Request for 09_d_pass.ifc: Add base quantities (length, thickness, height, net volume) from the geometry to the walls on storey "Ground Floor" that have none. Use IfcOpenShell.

First a look at what the model holds.

```python
import ifcopenshell
import ifcopenshell.util.element
import ifcopenshell.util.unit

model = ifcopenshell.open("09_d_pass.ifc")
print(model.schema)
for unit_type in ("LENGTHUNIT", "AREAUNIT", "VOLUMEUNIT"):
    print(unit_type, ifcopenshell.util.unit.calculate_unit_scale(model, unit_type))
storey = next(s for s in model.by_type("IfcBuildingStorey") if s.Name == "Ground Floor")
walls = [e for e in ifcopenshell.util.element.get_decomposition(storey) if e.is_a("IfcWall")]
for e in sorted(walls, key=lambda e: e.id()):
    print(e.id(), e.is_a(), e.Name, list(ifcopenshell.util.element.get_psets(e, qtos_only=True)), sep=" | ")
```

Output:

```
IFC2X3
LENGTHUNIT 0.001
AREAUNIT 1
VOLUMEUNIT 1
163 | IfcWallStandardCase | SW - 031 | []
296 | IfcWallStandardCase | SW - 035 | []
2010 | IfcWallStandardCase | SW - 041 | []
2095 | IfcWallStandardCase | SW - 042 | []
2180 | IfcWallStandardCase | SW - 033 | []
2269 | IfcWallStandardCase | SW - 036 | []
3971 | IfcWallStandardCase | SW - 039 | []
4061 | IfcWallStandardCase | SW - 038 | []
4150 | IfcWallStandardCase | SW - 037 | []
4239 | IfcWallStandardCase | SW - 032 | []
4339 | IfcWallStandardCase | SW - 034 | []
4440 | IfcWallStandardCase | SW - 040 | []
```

```python
import ifcopenshell
import ifcopenshell.api.pset
import ifcopenshell.geom
import ifcopenshell.util.element
import ifcopenshell.util.shape
import ifcopenshell.util.unit

model = ifcopenshell.open("09_d_pass.ifc")
unit_scale = ifcopenshell.util.unit.calculate_unit_scale(model)
volume_scale = ifcopenshell.util.unit.calculate_unit_scale(model, "VOLUMEUNIT")
settings = ifcopenshell.geom.settings()

storey = next(s for s in model.by_type("IfcBuildingStorey") if s.Name == "Ground Floor")
walls = [e for e in ifcopenshell.util.element.get_decomposition(storey) if e.is_a("IfcWall")]

for e in sorted(walls, key=lambda e: e.id()):
    if ifcopenshell.util.element.get_psets(e, qtos_only=True, should_inherit=False):
        continue
    # Geometry comes back in metres, in the element's own axes.
    shape = ifcopenshell.geom.create_shape(settings, e)
    values = {
        "Length": ifcopenshell.util.shape.get_x(shape.geometry) / unit_scale,
        "Width": ifcopenshell.util.shape.get_y(shape.geometry) / unit_scale,
        "Height": ifcopenshell.util.shape.get_z(shape.geometry) / unit_scale,
        "NetVolume": ifcopenshell.util.shape.get_volume(shape.geometry) / volume_scale,
    }
    qto = ifcopenshell.api.pset.add_qto(model, product=e, name="BaseQuantities")
    ifcopenshell.api.pset.edit_qto(model, qto=qto, properties=values)
    print(e.id(), {k: round(v, 3) for k, v in values.items()})

model.write("09_d_pass_v2.ifc")
```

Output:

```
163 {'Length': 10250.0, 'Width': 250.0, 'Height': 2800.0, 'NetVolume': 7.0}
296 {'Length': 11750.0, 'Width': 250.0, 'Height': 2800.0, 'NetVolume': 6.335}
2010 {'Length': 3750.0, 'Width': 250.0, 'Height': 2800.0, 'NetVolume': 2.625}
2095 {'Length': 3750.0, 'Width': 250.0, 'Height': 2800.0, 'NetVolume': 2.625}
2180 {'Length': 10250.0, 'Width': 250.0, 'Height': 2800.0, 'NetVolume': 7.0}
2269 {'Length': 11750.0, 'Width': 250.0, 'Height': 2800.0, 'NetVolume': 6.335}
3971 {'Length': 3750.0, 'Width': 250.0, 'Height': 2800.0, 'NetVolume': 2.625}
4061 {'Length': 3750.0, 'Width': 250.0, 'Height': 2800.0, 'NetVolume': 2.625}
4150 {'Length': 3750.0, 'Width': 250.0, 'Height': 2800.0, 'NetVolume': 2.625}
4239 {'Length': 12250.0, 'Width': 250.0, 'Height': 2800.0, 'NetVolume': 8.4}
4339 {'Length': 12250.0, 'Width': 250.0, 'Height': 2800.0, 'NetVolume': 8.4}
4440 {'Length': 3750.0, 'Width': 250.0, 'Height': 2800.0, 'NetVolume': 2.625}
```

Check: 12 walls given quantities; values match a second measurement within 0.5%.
